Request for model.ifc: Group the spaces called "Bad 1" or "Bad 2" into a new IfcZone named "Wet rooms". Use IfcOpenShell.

First a look at what the model holds.

```python
import ifcopenshell

model = ifcopenshell.open("model.ifc")
print(model.schema)
seen = {}
for space in model.by_type("IfcSpace"):
    seen[space.LongName] = seen.get(space.LongName, 0) + 1
for name, count in sorted(seen.items(), key=str):
    print(count, "x", name)
print("zones:", [z.Name for z in model.by_type("IfcZone")][:20])
```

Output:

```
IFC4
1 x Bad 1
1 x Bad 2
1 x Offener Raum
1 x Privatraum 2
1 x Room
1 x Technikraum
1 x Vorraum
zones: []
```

```python
import ifcopenshell
import ifcopenshell.api.group
import ifcopenshell.api.root

model = ifcopenshell.open("model.ifc")

names = {"Bad 1", "Bad 2"}
spaces = [s for s in model.by_type("IfcSpace") if s.LongName in names]

zone = ifcopenshell.api.root.create_entity(model, ifc_class="IfcZone", name="Wet rooms")
ifcopenshell.api.group.assign_group(model, products=spaces, group=zone)
print(len(spaces), "spaces in", zone.Name)

model.write("model-out.ifc")
```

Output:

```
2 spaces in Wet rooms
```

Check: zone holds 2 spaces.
